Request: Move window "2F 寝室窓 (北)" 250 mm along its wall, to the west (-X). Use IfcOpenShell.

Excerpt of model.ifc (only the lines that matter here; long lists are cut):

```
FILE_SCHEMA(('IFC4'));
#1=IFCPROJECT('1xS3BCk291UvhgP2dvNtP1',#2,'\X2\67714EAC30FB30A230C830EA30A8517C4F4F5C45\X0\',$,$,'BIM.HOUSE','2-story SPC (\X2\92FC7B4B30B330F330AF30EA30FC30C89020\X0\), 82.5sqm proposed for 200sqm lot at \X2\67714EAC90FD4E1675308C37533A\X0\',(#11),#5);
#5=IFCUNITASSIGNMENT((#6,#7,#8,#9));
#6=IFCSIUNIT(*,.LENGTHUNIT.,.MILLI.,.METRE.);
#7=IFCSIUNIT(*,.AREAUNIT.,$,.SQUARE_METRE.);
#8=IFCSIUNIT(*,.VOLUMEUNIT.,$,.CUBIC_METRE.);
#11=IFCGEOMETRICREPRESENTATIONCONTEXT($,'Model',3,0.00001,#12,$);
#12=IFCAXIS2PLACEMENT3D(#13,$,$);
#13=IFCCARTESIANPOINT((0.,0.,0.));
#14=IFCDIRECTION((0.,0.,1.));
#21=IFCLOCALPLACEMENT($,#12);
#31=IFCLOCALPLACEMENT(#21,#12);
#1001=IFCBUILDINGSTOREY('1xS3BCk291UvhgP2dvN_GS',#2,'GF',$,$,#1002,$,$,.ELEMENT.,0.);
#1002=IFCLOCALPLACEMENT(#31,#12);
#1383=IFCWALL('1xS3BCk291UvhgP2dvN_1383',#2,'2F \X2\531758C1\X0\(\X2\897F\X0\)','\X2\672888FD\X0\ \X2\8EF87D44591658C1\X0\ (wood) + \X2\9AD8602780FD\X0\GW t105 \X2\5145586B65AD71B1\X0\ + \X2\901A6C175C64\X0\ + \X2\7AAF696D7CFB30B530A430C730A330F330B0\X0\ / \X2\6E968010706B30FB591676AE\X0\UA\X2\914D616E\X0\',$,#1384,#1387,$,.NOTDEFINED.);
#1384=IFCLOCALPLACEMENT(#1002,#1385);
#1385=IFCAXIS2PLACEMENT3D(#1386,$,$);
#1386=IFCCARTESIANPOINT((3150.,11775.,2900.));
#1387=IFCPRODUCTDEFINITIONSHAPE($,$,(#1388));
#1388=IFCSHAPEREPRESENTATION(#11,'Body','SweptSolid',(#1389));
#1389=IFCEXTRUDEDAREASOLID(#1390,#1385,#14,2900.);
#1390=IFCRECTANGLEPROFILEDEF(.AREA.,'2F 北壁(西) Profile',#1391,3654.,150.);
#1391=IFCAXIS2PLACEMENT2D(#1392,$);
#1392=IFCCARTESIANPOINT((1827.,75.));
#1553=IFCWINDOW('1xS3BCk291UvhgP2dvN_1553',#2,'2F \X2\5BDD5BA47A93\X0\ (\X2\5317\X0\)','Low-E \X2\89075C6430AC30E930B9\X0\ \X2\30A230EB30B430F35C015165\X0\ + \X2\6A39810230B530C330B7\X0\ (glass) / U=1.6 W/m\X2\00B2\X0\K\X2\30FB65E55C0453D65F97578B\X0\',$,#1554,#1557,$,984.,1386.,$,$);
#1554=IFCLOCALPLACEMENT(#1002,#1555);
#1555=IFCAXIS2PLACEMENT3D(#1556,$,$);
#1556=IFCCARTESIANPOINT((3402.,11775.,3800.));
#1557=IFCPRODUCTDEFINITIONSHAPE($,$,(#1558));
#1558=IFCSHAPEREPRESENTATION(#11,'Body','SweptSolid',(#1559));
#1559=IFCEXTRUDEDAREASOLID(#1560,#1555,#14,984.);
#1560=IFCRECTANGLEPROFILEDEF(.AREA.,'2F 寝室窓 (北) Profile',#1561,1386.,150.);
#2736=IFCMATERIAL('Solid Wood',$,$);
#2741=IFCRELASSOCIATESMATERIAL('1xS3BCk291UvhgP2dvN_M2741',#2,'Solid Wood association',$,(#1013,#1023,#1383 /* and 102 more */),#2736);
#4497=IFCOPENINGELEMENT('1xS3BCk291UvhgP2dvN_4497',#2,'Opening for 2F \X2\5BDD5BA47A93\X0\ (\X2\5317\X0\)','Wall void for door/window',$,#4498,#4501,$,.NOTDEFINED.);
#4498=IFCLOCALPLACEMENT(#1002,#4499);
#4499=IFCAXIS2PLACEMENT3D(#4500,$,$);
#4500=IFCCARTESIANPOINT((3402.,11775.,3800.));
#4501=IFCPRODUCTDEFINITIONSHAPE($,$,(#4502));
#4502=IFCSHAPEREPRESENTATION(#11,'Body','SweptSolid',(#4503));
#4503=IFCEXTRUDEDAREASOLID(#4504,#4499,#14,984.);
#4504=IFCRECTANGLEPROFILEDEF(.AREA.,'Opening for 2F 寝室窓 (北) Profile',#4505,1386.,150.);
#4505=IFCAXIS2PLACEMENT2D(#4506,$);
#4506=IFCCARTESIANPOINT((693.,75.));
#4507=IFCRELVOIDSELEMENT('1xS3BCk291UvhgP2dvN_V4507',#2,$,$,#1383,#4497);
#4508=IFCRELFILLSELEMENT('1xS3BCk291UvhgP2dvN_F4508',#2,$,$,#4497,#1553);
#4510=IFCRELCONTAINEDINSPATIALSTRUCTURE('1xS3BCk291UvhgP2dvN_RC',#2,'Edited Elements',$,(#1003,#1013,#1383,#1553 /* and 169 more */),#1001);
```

```python
import ifcopenshell
import ifcopenshell.api.geometry
import ifcopenshell.util.placement
import ifcopenshell.util.unit

model = ifcopenshell.open("model.ifc")
unit_scale = ifcopenshell.util.unit.calculate_unit_scale(model)

window = model.by_guid("1xS3BCk291UvhgP2dvN_1553")
opening = window.FillsVoids[0].RelatingOpeningElement
wall = opening.VoidsElements[0].RelatingBuildingElement

wall_matrix = ifcopenshell.util.placement.get_local_placement(wall.ObjectPlacement)
shift = wall_matrix[:3, 0] * -0.25 / unit_scale
before = ifcopenshell.util.placement.get_local_placement(window.ObjectPlacement)[:3, 3].copy()

# The window is not placed relative to its opening, so move both.
for product in (opening, window):
    matrix = ifcopenshell.util.placement.get_local_placement(product.ObjectPlacement)
    matrix[:3, 3] += shift
    ifcopenshell.api.geometry.edit_object_placement(model, product=product, matrix=matrix, is_si=False)

after = ifcopenshell.util.placement.get_local_placement(window.ObjectPlacement)[:3, 3]
print("window moved by", (after - before).round(3) + 0.0)

model.write("model_edited.ifc")
```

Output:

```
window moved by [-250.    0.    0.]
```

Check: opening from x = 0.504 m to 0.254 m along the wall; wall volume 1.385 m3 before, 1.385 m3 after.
